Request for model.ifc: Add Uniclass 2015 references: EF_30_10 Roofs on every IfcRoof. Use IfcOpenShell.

First a look at what the model holds.

```python
import ifcopenshell

model = ifcopenshell.open("model.ifc")
print(model.schema)
print("classifications:", [c.Name for c in model.by_type("IfcClassification")])
for ifc_class in ("IfcDoor", "IfcRoof", "IfcStair", "IfcWall", "IfcWindow"):
    print(ifc_class, len(model.by_type(ifc_class)))
```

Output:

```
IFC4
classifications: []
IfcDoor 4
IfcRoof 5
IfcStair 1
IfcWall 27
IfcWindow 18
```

```python
import ifcopenshell
import ifcopenshell.api.classification

model = ifcopenshell.open("model.ifc")

system = ifcopenshell.api.classification.add_classification(model, classification="Uniclass 2015")

codes = {
    "IfcRoof": ("EF_30_10", "Roofs"),
}
for ifc_class, (code, name) in codes.items():
    products = model.by_type(ifc_class)
    ifcopenshell.api.classification.add_reference(
        model, products=products, classification=system, identification=code, name=name
    )
    print(code, len(products))

model.write("model_edited.ifc")
```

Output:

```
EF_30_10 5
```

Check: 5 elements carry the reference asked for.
